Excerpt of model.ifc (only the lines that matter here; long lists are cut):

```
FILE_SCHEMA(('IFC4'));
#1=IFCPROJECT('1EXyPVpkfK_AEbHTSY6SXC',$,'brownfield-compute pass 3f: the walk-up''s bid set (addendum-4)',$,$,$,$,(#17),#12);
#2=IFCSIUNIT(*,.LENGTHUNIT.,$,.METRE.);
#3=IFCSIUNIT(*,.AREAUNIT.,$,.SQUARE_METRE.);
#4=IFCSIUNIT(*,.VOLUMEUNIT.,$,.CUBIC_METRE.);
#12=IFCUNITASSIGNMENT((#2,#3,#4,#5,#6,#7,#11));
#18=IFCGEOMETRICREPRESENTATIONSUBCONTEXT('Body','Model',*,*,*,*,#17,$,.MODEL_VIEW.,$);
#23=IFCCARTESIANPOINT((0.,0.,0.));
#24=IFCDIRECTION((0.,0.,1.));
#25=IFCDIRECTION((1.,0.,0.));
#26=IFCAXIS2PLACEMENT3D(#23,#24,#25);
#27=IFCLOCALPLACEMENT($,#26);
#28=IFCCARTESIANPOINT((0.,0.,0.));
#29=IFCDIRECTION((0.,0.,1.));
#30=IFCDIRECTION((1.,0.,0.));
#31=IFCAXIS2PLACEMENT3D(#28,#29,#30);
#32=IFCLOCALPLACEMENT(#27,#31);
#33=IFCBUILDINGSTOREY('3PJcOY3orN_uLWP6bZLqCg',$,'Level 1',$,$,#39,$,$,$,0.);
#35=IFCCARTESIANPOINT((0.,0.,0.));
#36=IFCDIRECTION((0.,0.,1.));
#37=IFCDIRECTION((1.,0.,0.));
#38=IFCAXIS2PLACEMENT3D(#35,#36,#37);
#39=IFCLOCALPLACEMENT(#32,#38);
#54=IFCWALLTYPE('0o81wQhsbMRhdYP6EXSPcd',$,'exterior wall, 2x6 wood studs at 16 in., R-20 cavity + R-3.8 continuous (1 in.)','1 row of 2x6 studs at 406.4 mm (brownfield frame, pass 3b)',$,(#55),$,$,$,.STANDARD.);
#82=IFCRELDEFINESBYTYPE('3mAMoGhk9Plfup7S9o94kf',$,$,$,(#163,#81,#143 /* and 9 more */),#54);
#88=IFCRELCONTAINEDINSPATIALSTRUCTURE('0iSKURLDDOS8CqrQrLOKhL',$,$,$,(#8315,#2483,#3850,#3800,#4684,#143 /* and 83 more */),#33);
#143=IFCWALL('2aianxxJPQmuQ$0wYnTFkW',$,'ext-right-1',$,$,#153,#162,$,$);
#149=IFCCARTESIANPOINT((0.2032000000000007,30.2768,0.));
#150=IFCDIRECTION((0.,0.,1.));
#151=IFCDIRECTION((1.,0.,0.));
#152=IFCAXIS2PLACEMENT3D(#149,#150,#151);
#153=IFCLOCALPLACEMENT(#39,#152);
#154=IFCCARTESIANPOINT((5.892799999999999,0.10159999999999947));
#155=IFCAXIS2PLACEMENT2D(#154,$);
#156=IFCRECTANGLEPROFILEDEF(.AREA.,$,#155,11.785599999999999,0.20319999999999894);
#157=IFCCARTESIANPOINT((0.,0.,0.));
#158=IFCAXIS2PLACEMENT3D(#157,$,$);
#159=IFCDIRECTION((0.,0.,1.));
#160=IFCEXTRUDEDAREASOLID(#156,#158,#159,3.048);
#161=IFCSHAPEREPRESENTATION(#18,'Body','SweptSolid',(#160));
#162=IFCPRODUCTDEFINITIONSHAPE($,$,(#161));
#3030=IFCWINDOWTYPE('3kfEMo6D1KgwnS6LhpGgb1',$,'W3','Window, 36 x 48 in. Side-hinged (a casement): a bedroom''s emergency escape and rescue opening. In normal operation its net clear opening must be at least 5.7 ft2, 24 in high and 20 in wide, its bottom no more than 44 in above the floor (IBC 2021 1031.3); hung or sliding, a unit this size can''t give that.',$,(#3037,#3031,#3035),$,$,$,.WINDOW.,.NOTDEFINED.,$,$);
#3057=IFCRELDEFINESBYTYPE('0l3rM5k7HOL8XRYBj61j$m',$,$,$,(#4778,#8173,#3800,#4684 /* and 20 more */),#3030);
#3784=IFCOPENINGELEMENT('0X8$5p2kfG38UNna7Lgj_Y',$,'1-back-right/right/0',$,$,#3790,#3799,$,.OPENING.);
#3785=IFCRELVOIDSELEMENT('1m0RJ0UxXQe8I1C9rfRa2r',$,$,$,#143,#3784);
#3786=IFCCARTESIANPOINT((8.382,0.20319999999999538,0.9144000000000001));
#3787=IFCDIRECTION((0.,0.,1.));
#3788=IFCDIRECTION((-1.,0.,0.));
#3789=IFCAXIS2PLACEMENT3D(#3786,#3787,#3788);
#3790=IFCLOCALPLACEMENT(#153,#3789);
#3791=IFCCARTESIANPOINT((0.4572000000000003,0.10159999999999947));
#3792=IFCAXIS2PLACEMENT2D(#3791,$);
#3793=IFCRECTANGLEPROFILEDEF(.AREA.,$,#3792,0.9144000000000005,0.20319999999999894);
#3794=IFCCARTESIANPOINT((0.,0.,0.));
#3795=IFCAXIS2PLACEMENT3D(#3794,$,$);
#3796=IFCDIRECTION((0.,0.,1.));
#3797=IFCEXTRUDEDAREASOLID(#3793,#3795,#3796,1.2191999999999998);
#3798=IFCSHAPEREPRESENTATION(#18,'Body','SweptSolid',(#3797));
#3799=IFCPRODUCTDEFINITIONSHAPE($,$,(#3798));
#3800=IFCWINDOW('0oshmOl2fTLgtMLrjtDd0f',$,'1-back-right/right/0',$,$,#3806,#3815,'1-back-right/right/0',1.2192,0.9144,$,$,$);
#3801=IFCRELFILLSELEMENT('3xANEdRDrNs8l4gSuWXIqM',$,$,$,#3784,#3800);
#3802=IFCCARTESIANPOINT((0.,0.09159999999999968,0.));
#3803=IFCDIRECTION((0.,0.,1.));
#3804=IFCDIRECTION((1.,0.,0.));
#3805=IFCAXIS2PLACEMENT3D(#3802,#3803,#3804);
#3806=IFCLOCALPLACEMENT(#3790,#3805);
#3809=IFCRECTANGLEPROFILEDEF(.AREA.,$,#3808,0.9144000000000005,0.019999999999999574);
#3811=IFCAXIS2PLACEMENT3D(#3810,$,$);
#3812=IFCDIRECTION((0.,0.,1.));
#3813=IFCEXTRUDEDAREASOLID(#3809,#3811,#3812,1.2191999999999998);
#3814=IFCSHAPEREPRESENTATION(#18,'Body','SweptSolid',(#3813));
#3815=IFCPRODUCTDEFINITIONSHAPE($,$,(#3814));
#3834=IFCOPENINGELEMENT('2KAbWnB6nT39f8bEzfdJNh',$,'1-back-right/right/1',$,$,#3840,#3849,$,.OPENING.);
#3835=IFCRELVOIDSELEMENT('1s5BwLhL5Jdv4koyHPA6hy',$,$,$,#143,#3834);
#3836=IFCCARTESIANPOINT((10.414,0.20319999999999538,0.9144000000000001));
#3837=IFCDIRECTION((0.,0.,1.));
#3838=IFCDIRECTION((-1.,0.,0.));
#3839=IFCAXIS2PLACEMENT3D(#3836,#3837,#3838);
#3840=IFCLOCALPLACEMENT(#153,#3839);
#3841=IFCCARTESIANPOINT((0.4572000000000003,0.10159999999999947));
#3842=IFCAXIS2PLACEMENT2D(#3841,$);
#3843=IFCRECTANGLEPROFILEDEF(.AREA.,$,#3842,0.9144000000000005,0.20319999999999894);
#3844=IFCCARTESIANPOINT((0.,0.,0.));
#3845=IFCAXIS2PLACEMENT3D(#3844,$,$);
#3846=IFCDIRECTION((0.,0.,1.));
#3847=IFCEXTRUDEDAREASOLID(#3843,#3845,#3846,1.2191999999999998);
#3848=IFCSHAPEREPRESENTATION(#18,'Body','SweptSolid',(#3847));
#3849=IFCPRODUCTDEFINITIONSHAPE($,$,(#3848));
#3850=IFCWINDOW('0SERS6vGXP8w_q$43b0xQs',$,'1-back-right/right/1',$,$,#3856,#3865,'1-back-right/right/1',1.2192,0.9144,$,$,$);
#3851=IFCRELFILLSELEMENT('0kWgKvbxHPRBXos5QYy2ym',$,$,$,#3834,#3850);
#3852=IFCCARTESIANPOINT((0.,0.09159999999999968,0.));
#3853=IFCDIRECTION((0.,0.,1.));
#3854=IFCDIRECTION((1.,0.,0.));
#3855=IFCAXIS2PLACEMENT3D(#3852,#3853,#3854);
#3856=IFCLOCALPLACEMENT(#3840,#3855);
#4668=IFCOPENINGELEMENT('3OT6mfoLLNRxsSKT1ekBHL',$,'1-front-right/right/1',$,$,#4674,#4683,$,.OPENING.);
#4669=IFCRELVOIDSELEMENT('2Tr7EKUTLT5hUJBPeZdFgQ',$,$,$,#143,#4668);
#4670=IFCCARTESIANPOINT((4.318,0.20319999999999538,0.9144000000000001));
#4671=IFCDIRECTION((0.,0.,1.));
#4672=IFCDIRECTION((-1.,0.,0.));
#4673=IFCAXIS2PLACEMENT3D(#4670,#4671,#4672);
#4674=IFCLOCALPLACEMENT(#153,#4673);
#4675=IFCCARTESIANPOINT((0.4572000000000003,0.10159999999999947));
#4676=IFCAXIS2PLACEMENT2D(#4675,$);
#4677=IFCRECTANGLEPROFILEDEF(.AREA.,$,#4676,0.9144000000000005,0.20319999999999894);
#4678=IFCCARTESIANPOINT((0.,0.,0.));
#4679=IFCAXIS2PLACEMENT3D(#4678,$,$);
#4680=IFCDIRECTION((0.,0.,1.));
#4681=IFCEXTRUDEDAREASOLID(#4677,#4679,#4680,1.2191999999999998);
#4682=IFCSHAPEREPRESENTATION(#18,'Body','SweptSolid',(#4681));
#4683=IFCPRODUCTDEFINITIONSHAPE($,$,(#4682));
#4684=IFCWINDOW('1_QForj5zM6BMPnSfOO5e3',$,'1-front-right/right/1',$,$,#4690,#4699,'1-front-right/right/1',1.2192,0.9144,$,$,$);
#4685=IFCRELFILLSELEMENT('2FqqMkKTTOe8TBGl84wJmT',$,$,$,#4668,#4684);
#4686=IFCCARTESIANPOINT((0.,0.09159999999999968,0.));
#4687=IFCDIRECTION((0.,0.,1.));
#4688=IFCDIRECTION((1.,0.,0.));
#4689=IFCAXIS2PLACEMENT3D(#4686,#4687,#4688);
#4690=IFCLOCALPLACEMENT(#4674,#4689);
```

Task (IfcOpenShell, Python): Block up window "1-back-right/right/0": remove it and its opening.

```python
import ifcopenshell
import ifcopenshell.api.feature
import ifcopenshell.api.root
import ifcopenshell.geom
import ifcopenshell.util.shape

model = ifcopenshell.open("model.ifc")
settings = ifcopenshell.geom.settings()


def volume(element):
    """Net volume in cubic metres, openings subtracted."""
    shape = ifcopenshell.geom.create_shape(settings, element)
    return ifcopenshell.util.shape.get_volume(shape.geometry)


window = model.by_id(3800)
opening = window.FillsVoids[0].RelatingOpeningElement
wall = opening.VoidsElements[0].RelatingBuildingElement
before = volume(wall)

ifcopenshell.api.root.remove_product(model, product=window)
ifcopenshell.api.feature.remove_feature(model, feature=opening)

after = volume(wall)

print(f"wall volume {before:.3f} -> {after:.3f} m3")

model.write("model_edited.ifc")
```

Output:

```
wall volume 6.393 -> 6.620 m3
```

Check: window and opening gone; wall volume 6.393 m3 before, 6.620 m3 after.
